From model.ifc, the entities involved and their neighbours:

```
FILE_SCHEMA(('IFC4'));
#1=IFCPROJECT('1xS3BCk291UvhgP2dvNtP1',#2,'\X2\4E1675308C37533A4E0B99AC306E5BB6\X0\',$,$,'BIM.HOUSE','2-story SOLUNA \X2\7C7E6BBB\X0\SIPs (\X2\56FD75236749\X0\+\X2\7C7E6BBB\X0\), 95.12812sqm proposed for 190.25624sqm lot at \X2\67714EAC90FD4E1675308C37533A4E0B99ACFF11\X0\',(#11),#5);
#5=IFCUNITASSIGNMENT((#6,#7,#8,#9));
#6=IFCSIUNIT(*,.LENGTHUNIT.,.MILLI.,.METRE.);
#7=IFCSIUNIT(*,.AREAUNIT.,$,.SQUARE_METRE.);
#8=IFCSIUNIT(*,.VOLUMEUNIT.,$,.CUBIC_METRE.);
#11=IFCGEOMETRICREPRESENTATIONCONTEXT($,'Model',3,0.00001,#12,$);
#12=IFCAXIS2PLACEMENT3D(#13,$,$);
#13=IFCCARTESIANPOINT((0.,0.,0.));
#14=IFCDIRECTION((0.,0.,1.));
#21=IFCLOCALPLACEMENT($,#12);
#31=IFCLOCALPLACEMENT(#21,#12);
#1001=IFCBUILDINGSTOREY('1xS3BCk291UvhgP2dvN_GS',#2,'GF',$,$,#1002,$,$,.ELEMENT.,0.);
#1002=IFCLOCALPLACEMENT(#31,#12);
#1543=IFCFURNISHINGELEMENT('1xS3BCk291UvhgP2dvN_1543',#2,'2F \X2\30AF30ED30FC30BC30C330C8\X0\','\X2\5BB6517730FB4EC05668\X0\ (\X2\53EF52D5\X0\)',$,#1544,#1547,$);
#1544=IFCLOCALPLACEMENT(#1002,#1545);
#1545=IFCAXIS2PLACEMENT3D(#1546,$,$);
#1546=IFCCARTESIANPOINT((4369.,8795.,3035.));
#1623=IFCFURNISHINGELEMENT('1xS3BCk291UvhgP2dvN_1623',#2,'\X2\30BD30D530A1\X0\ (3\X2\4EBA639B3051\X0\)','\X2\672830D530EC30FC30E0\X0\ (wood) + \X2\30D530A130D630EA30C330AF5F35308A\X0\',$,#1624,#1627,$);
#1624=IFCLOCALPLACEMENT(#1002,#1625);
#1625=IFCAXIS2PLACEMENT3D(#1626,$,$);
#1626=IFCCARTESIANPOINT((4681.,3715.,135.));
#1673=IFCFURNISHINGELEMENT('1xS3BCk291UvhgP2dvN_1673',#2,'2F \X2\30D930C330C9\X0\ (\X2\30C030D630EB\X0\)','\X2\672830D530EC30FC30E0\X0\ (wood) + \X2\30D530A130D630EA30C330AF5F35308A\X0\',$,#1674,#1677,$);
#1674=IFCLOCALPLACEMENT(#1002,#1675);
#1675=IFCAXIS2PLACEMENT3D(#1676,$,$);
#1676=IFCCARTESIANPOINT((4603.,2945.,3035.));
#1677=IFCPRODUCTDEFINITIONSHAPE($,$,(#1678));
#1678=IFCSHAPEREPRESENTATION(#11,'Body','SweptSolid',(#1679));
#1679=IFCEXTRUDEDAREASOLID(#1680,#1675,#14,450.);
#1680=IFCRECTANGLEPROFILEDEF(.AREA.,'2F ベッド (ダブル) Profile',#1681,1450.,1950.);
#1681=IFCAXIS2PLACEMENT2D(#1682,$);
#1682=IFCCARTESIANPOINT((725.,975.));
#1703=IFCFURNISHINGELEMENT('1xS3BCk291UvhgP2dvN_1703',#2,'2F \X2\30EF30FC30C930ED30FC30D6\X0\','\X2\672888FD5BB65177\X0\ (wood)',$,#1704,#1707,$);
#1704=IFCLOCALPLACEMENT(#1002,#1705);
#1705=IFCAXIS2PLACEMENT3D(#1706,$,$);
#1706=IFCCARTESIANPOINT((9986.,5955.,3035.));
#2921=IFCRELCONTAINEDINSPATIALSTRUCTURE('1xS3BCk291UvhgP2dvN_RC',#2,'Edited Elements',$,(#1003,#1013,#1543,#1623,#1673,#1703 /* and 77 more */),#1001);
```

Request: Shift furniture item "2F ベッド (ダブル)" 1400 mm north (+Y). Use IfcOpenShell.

```python
import ifcopenshell
import ifcopenshell.api.geometry
import ifcopenshell.util.placement

model = ifcopenshell.open("model.ifc")

item = model.by_guid("1xS3BCk291UvhgP2dvN_1673")
matrix = ifcopenshell.util.placement.get_local_placement(item.ObjectPlacement)
matrix[1, 3] += 1400.0
ifcopenshell.api.geometry.edit_object_placement(model, product=item, matrix=matrix, is_si=False)

print(ifcopenshell.util.placement.get_local_placement(item.ObjectPlacement).round(3) + 0.0)

model.write("model-out.ifc")
```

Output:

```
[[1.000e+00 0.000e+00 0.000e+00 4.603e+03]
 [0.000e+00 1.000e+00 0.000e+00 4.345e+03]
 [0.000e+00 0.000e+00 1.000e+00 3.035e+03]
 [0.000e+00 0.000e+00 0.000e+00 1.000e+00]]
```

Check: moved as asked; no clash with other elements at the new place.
